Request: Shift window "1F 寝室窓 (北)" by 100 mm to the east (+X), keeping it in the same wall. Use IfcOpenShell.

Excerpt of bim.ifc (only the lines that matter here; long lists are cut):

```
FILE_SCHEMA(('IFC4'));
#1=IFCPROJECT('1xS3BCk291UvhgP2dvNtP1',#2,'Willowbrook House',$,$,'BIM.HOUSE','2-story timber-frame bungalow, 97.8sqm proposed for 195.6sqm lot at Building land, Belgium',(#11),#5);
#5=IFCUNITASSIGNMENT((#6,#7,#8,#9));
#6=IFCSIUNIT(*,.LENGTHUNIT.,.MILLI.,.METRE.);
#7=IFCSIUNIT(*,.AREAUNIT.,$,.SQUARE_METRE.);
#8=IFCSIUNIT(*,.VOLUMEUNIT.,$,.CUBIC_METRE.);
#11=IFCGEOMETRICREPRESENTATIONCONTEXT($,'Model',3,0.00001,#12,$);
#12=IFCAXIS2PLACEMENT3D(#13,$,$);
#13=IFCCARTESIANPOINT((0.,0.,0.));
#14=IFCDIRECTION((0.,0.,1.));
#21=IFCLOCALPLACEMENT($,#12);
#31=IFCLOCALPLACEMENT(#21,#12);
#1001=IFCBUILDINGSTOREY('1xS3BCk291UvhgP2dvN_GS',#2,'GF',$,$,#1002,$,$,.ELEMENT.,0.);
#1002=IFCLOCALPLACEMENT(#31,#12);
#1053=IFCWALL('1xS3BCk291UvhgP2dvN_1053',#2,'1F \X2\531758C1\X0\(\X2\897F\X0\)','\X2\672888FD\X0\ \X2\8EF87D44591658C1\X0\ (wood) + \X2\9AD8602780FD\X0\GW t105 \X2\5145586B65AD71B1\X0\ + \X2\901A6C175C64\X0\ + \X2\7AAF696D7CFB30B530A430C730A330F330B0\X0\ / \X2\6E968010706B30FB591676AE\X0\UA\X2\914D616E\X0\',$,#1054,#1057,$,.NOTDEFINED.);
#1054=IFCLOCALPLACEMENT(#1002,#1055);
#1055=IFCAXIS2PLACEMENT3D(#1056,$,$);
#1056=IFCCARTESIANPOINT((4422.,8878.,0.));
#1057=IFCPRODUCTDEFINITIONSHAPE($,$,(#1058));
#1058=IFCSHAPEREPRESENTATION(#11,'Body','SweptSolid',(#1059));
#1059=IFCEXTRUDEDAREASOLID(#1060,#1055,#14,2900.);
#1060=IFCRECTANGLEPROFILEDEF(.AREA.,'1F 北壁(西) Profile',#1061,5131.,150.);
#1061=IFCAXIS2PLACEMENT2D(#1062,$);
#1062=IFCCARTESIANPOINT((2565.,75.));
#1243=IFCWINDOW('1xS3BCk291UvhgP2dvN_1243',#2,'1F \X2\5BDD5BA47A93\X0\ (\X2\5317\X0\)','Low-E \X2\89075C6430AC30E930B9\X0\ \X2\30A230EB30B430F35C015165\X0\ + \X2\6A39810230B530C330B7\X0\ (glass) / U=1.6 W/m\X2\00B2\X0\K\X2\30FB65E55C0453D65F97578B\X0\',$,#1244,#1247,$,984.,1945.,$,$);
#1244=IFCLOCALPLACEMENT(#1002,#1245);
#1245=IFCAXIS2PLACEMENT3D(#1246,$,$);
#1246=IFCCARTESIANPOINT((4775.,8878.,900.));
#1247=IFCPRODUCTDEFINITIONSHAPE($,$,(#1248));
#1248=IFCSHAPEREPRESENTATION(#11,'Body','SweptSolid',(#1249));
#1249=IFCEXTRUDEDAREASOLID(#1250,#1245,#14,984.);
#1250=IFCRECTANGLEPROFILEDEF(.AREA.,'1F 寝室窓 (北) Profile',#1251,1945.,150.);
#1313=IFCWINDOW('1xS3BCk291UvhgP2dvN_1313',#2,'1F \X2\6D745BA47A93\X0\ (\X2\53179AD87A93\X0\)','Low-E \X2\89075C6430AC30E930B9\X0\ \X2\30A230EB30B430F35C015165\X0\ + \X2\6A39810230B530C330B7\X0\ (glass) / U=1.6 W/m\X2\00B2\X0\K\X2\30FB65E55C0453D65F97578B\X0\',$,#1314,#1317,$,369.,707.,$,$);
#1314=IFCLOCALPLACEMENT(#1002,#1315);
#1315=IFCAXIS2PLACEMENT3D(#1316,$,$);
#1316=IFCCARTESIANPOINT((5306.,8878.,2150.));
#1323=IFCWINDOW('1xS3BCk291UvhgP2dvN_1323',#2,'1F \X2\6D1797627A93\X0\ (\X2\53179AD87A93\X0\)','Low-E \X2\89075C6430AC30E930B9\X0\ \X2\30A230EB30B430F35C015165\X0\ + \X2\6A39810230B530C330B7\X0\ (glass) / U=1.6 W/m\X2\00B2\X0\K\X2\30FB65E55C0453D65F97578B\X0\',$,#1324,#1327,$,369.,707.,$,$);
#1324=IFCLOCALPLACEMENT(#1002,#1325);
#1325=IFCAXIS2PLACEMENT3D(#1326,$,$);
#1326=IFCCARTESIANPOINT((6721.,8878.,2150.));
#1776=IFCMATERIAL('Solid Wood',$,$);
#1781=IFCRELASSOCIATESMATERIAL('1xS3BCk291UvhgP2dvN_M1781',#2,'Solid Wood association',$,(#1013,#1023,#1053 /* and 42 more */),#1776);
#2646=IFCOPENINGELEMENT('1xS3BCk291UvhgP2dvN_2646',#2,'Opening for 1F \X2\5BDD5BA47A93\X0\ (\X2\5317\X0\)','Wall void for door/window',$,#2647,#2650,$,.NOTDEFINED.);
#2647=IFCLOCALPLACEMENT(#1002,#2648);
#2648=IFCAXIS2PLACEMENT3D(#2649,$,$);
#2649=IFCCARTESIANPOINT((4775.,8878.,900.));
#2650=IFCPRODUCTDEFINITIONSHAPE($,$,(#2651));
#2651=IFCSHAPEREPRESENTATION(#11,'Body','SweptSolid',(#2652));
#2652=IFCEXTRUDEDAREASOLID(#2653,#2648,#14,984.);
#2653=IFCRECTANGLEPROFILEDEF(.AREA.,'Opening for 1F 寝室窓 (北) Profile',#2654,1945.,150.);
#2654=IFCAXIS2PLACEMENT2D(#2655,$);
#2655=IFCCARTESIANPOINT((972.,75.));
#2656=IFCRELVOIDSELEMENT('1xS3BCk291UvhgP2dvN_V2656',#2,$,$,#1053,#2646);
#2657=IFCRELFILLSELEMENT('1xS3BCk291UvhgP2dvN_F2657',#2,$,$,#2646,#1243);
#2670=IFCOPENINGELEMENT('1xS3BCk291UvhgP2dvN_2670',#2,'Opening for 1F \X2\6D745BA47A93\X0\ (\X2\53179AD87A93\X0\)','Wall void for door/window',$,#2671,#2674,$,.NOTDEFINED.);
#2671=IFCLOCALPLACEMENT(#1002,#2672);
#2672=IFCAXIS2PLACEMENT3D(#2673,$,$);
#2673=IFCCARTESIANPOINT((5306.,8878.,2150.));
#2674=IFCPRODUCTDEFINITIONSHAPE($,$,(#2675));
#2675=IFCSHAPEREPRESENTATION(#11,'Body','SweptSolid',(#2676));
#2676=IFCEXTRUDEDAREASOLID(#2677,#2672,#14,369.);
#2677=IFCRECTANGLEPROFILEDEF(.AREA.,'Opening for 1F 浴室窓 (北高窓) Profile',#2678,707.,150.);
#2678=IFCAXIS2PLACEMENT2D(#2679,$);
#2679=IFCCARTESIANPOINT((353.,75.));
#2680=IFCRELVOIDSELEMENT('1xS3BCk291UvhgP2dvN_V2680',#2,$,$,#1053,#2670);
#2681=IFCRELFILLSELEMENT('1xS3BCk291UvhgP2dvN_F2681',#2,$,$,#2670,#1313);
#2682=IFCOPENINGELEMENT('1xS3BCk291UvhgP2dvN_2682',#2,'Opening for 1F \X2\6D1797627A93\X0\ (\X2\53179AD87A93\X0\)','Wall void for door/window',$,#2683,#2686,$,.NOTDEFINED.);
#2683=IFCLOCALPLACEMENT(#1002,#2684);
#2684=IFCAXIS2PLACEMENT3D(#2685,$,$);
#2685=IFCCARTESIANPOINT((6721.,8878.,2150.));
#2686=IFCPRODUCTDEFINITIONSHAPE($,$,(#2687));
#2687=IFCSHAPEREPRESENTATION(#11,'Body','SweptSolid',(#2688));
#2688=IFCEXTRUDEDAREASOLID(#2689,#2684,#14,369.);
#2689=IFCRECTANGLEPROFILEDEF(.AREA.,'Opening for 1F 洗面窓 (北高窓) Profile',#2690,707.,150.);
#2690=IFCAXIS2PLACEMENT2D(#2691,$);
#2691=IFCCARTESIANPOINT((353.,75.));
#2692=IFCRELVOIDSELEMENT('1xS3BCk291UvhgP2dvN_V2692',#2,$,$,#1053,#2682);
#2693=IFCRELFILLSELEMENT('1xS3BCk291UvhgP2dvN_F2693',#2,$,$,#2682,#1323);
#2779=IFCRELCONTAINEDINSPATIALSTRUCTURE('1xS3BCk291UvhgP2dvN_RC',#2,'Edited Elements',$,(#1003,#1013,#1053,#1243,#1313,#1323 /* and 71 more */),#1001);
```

```python
import ifcopenshell
import ifcopenshell.api.geometry
import ifcopenshell.util.placement

model = ifcopenshell.open("bim.ifc")

window = model.by_guid("1xS3BCk291UvhgP2dvN_1243")
opening = window.FillsVoids[0].RelatingOpeningElement
wall = opening.VoidsElements[0].RelatingBuildingElement

wall_matrix = ifcopenshell.util.placement.get_local_placement(wall.ObjectPlacement)
shift = wall_matrix[:3, 0] * 100.0
before = ifcopenshell.util.placement.get_local_placement(window.ObjectPlacement)[:3, 3].copy()

# The window is not placed relative to its opening, so move both.
for product in (opening, window):
    matrix = ifcopenshell.util.placement.get_local_placement(product.ObjectPlacement)
    matrix[:3, 3] += shift
    ifcopenshell.api.geometry.edit_object_placement(model, product=product, matrix=matrix, is_si=False)

after = ifcopenshell.util.placement.get_local_placement(window.ObjectPlacement)[:3, 3]
print("window moved by", (after - before).round(3) + 0.0)

model.write("bim_rev.ifc")
```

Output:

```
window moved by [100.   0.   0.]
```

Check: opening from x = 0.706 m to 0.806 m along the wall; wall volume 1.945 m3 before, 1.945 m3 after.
